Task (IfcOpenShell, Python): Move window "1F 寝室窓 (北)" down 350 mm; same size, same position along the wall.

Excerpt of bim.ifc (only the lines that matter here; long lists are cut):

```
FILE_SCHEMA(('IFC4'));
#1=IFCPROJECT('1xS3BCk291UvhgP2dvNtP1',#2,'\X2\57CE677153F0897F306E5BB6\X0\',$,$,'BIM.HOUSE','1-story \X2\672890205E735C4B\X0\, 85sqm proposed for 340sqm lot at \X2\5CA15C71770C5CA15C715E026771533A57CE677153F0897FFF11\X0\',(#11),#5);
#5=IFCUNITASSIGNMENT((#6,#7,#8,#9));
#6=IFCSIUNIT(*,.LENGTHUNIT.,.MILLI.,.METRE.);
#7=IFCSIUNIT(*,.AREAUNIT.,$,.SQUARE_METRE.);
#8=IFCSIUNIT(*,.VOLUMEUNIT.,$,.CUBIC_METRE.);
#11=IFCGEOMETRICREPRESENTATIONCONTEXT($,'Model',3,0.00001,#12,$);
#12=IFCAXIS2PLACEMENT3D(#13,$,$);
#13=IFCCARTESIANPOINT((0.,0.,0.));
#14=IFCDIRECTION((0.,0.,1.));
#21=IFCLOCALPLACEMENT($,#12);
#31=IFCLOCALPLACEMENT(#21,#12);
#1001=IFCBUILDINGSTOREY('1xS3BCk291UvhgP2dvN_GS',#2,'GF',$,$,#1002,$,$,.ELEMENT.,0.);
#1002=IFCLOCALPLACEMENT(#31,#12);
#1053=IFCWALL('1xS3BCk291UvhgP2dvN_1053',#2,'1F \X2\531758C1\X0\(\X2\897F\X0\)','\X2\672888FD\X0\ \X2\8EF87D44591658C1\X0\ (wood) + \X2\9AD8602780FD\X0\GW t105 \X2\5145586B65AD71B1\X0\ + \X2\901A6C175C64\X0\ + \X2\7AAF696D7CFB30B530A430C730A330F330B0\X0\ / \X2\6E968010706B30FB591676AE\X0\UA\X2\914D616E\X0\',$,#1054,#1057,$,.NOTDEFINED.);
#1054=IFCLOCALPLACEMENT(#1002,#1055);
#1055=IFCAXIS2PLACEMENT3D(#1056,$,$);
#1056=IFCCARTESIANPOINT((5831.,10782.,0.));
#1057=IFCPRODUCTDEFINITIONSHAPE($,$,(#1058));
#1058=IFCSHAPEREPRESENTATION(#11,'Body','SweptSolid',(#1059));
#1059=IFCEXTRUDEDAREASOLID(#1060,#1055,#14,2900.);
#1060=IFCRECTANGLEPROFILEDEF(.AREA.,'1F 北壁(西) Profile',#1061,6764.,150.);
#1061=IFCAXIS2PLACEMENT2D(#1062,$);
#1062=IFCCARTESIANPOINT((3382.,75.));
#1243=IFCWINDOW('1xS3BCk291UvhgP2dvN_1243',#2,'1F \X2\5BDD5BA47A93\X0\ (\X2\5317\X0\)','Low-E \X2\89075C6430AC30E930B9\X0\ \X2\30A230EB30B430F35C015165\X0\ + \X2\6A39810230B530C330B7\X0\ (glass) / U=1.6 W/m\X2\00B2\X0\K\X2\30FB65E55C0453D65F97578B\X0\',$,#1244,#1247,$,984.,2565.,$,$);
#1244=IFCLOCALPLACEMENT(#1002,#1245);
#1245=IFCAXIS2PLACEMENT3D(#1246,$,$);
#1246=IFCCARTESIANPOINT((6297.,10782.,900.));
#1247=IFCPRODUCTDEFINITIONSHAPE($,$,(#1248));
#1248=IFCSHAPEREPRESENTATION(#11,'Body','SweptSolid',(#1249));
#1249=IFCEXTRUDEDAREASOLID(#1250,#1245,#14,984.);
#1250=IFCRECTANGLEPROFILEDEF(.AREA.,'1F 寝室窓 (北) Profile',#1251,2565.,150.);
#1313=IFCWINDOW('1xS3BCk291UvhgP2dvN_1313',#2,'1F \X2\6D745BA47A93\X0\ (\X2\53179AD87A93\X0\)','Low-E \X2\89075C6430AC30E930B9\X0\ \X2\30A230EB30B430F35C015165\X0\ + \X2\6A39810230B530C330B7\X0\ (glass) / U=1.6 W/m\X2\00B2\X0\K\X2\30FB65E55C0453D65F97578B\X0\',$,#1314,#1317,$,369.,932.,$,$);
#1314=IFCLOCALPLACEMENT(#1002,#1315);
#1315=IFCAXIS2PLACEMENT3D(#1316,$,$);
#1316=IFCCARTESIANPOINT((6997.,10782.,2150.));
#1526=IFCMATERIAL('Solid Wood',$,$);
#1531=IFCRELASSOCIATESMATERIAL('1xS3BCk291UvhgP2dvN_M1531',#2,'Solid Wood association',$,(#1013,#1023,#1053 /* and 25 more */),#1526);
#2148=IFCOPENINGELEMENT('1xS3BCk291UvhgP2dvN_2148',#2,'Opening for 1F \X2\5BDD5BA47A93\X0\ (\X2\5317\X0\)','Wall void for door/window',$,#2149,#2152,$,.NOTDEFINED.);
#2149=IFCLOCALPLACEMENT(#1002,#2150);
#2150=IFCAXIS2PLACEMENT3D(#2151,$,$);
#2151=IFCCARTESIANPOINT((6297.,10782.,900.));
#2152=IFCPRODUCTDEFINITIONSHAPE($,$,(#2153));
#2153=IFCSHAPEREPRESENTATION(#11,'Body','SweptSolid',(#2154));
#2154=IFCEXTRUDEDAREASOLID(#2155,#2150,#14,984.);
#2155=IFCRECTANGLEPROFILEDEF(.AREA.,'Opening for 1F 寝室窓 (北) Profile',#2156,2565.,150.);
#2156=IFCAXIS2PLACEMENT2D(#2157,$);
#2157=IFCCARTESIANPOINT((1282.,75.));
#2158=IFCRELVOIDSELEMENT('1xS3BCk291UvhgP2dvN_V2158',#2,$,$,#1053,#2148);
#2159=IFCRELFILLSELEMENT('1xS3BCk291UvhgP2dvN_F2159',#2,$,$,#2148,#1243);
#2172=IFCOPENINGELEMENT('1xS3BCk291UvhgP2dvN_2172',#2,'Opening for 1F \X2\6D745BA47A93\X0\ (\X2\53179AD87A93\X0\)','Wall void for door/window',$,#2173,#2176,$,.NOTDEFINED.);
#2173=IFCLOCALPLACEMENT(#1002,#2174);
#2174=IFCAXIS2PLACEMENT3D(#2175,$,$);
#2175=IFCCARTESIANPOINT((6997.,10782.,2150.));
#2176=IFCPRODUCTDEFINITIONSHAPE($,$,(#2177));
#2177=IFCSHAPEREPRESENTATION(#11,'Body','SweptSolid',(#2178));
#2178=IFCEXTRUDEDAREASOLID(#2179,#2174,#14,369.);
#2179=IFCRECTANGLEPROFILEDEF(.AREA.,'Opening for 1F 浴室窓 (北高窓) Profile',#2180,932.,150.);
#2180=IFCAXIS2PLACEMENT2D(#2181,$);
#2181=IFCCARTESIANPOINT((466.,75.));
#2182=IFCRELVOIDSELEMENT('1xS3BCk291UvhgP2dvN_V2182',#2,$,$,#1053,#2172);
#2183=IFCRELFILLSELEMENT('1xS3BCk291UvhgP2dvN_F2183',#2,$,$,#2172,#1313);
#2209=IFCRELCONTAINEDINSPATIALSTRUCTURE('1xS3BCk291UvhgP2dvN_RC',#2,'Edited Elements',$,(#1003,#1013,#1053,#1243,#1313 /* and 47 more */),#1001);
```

```python
import numpy as np
import ifcopenshell
import ifcopenshell.api.geometry
import ifcopenshell.util.placement
import ifcopenshell.util.unit

model = ifcopenshell.open("bim.ifc")
unit_scale = ifcopenshell.util.unit.calculate_unit_scale(model)

window = model.by_id(1243)
opening = window.FillsVoids[0].RelatingOpeningElement
dz = -350.0

shift = np.array([0.0, 0.0, dz])
# The window is not placed relative to its opening, so move both.
for product in (opening, window):
    matrix = ifcopenshell.util.placement.get_local_placement(product.ObjectPlacement)
    matrix[:3, 3] += shift
    ifcopenshell.api.geometry.edit_object_placement(model, product=product, matrix=matrix, is_si=False)

print(f"moved by {dz * unit_scale:+.3f} m")

model.write("bim_v2.ifc")
```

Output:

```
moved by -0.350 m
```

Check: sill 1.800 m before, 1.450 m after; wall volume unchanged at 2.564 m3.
